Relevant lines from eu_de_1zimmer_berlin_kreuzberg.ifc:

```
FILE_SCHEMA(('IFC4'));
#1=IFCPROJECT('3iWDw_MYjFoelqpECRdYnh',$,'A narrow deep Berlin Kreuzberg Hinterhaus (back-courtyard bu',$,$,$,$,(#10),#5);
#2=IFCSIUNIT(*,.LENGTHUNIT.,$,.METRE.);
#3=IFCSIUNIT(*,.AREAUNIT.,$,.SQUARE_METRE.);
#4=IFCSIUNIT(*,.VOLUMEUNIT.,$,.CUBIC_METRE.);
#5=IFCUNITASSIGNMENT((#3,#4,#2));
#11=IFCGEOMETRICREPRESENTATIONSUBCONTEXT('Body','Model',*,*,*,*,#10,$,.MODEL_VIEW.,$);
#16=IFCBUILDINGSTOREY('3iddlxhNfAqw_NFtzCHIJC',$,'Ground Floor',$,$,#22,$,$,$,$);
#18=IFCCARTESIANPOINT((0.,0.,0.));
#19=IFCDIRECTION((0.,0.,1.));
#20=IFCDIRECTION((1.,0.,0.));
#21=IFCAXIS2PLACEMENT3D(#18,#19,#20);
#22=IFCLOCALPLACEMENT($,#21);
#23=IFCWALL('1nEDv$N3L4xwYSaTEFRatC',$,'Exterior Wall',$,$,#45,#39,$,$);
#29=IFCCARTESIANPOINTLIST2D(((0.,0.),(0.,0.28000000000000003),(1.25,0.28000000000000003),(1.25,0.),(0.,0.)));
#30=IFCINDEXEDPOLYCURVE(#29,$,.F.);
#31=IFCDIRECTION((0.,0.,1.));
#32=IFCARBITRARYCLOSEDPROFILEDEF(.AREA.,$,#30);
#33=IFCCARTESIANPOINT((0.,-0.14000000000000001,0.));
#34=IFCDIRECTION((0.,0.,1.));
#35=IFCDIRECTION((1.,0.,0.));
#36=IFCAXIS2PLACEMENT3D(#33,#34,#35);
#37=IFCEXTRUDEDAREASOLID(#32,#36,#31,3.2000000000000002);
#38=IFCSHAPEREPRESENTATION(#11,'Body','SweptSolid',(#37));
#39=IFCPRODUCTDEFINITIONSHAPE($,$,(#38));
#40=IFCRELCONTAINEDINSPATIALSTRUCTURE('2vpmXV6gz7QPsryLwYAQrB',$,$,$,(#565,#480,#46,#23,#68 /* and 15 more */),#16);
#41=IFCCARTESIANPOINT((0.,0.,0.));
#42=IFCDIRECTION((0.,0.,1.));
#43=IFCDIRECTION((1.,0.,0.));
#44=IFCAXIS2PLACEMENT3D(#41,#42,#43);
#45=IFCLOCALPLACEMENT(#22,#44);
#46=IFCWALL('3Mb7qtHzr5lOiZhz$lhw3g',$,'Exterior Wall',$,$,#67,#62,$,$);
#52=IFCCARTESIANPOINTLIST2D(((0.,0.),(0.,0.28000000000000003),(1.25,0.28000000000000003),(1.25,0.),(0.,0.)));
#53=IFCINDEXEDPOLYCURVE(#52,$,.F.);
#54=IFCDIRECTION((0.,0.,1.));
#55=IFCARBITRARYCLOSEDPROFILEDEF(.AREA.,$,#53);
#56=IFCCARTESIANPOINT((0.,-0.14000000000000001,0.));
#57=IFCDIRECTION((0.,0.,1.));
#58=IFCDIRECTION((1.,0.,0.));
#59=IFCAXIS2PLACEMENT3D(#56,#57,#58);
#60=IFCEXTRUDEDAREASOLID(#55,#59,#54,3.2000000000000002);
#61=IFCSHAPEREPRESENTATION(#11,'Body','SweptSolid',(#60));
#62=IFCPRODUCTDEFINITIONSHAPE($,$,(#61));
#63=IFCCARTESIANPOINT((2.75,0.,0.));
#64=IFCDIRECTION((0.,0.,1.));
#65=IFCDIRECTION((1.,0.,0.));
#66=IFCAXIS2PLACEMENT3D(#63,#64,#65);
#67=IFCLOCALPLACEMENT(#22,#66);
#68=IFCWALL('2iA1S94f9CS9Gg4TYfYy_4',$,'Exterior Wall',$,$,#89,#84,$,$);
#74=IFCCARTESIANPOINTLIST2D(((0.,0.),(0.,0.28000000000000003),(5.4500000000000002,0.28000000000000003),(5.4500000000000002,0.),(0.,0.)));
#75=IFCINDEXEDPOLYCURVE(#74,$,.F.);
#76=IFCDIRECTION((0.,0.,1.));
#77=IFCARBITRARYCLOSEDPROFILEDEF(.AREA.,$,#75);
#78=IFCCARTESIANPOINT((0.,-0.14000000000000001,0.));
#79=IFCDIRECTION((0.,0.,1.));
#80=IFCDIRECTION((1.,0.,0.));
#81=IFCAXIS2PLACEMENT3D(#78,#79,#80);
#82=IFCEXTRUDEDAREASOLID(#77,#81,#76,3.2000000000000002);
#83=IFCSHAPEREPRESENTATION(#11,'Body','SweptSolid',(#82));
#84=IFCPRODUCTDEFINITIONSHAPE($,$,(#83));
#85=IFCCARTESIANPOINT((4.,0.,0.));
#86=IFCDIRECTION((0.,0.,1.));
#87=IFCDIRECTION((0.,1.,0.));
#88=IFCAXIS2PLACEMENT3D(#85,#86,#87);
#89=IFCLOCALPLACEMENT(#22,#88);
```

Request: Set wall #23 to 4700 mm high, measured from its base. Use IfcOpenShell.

```python
import ifcopenshell
import ifcopenshell.geom
import ifcopenshell.util.representation
import ifcopenshell.util.shape

model = ifcopenshell.open("eu_de_1zimmer_berlin_kreuzberg.ifc")
settings = ifcopenshell.geom.settings()


def volume(element):
    """Net volume in cubic metres, openings subtracted."""
    shape = ifcopenshell.geom.create_shape(settings, element)
    return ifcopenshell.util.shape.get_volume(shape.geometry)


wall = model.by_id(23)
before = volume(wall)

body = ifcopenshell.util.representation.get_representation(wall, "Model", "Body")
solid = body.Items[0]
old_height = solid.Depth
solid.Depth = 4.7
after = volume(wall)

print(f"height {old_height:g} -> {solid.Depth:g}, volume {before:.3f} -> {after:.3f} m3")

model.write("eu_de_1zimmer_berlin_kreuzberg-out.ifc")
```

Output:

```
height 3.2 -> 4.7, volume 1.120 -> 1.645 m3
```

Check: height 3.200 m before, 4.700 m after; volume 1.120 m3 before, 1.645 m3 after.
